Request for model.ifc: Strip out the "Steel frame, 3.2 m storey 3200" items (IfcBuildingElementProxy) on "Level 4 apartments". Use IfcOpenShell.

First a look at what the model holds.

```python
import ifcopenshell
import ifcopenshell.util.element

model = ifcopenshell.open("model.ifc")
print(model.schema)
storey = next(s for s in model.by_type("IfcBuildingStorey") if s.Name == "Level 4 apartments")
proxies = [e for e in ifcopenshell.util.element.get_decomposition(storey) if e.is_a("IfcBuildingElementProxy")]
seen = {}
for e in proxies:
    element_type = ifcopenshell.util.element.get_type(e)
    name = element_type.Name if element_type not in (None, e) else None
    seen[name] = seen.get(name, 0) + 1
for name, count in sorted(seen.items(), key=str):
    print(count, "x", name)
```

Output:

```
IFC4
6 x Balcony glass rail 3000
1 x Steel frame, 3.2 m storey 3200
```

```python
import ifcopenshell
import ifcopenshell.api.root
import ifcopenshell.util.element

model = ifcopenshell.open("model.ifc")

storey = next(s for s in model.by_type("IfcBuildingStorey") if s.Name == "Level 4 apartments")
proxies = [e for e in ifcopenshell.util.element.get_decomposition(storey) if e.is_a("IfcBuildingElementProxy")]
targets = [e for e in proxies if (t := ifcopenshell.util.element.get_type(e)) not in (None, e) and t.Name == "Steel frame, 3.2 m storey 3200"]

for e in targets:
    ifcopenshell.api.root.remove_product(model, product=e)
print(len(targets), "removed")

model.write("model-out.ifc")
```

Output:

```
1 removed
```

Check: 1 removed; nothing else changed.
